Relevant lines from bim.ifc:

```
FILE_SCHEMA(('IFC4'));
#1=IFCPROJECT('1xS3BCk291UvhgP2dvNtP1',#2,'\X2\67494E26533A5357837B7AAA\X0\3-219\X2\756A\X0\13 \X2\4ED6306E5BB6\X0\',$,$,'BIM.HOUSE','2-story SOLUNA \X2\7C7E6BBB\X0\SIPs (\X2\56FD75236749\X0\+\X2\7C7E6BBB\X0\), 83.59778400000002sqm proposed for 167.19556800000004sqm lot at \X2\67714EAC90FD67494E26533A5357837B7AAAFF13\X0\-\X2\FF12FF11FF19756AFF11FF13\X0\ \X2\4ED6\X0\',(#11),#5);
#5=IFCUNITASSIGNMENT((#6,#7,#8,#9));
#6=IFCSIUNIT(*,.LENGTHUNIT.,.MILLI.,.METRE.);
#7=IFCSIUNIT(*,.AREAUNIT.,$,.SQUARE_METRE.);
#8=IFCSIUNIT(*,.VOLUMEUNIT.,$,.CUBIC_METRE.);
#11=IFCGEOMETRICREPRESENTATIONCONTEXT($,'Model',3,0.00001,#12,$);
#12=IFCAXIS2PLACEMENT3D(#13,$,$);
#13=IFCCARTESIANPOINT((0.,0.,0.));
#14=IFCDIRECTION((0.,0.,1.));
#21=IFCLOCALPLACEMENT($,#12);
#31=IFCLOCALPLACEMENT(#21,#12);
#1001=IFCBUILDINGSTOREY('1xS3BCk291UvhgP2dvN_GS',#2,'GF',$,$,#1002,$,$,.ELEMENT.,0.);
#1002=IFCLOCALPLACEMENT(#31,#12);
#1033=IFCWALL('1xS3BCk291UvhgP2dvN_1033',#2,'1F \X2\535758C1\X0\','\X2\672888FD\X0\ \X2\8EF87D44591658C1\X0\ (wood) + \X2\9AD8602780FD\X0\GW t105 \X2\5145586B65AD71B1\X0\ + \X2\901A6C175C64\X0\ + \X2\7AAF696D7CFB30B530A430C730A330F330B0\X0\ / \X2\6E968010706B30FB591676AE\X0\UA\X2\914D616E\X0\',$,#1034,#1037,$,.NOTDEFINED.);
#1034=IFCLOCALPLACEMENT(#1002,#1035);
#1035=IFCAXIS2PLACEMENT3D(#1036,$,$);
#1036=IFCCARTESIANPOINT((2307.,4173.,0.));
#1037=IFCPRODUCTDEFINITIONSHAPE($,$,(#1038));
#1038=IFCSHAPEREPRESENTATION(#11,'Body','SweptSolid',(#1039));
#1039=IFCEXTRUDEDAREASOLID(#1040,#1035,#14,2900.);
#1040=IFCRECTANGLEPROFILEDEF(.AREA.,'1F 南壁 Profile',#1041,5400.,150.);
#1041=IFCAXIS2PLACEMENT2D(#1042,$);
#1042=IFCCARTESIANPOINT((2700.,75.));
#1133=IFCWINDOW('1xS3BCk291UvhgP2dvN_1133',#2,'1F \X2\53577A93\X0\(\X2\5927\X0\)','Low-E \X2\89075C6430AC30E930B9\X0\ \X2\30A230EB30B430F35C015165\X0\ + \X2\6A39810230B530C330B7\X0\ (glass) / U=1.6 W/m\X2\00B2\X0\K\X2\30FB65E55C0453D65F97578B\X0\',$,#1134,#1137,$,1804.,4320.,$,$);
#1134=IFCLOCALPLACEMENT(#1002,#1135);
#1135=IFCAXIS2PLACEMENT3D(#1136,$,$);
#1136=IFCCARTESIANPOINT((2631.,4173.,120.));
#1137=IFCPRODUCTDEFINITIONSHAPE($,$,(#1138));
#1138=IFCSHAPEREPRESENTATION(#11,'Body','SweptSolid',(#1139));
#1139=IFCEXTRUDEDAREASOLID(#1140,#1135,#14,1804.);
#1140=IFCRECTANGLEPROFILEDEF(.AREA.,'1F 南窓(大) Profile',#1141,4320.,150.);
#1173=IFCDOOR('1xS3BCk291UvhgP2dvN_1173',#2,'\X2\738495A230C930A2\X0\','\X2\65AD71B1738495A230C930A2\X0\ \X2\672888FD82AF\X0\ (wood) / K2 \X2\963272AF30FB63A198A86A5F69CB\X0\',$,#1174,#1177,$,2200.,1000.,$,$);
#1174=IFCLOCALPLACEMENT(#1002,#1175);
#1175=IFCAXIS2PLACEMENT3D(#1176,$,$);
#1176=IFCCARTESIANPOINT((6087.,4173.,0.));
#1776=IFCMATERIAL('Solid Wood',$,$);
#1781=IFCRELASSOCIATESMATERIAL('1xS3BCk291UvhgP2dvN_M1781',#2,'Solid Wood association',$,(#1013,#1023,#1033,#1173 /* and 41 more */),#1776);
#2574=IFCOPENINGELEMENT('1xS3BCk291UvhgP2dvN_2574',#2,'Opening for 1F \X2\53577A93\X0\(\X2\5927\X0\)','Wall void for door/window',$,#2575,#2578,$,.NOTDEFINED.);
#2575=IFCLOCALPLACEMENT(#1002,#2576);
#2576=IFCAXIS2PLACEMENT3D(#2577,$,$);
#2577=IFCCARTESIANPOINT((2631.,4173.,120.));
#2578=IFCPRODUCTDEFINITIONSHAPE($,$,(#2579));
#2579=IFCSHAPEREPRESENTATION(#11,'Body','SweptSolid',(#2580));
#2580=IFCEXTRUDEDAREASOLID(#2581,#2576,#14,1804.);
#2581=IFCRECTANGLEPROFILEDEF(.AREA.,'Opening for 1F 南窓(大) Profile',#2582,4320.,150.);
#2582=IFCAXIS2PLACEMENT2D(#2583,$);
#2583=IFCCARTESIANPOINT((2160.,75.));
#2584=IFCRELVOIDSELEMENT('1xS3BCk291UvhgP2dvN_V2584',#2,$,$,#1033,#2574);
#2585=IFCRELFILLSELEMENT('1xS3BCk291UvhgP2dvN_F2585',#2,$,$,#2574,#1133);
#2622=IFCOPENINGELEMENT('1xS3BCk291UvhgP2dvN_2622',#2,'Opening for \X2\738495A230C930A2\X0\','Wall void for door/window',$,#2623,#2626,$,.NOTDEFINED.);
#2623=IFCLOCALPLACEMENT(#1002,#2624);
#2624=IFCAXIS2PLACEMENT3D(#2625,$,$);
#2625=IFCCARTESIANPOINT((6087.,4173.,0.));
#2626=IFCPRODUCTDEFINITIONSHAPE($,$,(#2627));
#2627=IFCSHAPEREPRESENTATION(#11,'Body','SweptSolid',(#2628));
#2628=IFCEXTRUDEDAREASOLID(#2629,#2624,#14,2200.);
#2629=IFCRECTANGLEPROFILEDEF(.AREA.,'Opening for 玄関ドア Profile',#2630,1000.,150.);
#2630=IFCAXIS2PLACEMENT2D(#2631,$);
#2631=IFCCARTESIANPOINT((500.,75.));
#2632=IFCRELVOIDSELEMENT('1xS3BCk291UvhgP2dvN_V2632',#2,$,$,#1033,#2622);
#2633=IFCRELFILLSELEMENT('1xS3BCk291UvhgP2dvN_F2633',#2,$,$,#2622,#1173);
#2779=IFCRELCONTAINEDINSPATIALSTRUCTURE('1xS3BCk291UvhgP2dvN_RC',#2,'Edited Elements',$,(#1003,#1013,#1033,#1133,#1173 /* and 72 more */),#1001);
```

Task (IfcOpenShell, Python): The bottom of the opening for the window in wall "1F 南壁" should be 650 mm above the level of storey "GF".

```python
import numpy as np
import ifcopenshell
import ifcopenshell.api.geometry
import ifcopenshell.geom
import ifcopenshell.util.element
import ifcopenshell.util.placement
import ifcopenshell.util.shape
import ifcopenshell.util.unit

model = ifcopenshell.open("bim.ifc")
unit_scale = ifcopenshell.util.unit.calculate_unit_scale(model)

window = model.by_guid("1xS3BCk291UvhgP2dvN_1133")
opening = window.FillsVoids[0].RelatingOpeningElement
storey = ifcopenshell.util.element.get_container(window, ifc_class="IfcBuildingStorey")
level = ifcopenshell.util.placement.get_local_placement(storey.ObjectPlacement)[2, 3]

# The opening's origin need not be at the sill, so measure its lowest point.
shape = ifcopenshell.geom.create_shape(ifcopenshell.geom.settings(), opening)
bottom = ifcopenshell.util.shape.get_shape_bottom_elevation(shape, shape.geometry) / unit_scale
dz = level + 0.65 / unit_scale - bottom

shift = np.array([0.0, 0.0, dz])
# The window is not placed relative to its opening, so move both.
for product in (opening, window):
    matrix = ifcopenshell.util.placement.get_local_placement(product.ObjectPlacement)
    matrix[:3, 3] += shift
    ifcopenshell.api.geometry.edit_object_placement(model, product=product, matrix=matrix, is_si=False)

print(f"moved by {dz * unit_scale:+.3f} m")

model.write("bim_v2.ifc")
```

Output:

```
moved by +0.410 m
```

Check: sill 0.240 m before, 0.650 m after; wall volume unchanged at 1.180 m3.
